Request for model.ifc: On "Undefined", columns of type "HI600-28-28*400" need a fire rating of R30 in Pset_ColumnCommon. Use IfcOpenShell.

First a look at what the model holds.

```python
import ifcopenshell
import ifcopenshell.util.element

model = ifcopenshell.open("model.ifc")
print(model.schema)
storey = next(s for s in model.by_type("IfcBuildingStorey") if s.Name == "Undefined")
columns = [e for e in ifcopenshell.util.element.get_decomposition(storey) if e.is_a("IfcColumn")]
seen = {}
for e in columns:
    element_type = ifcopenshell.util.element.get_type(e)
    key = (element_type.Name if element_type != e and element_type else None, ifcopenshell.util.element.get_pset(e, "Pset_ColumnCommon", "FireRating"))
    seen[key] = seen.get(key, 0) + 1
for (name, value), count in sorted(seen.items(), key=str):
    print(count, "x", name, "|", value)
```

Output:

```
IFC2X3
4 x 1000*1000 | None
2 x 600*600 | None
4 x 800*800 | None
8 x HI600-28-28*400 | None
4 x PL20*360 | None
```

```python
import ifcopenshell
import ifcopenshell.api.pset
import ifcopenshell.util.element

model = ifcopenshell.open("model.ifc")

storey = next(s for s in model.by_type("IfcBuildingStorey") if s.Name == "Undefined")
columns = [e for e in ifcopenshell.util.element.get_decomposition(storey) if e.is_a("IfcColumn")]

count = 0
for e in columns:
    element_type = ifcopenshell.util.element.get_type(e)
    if element_type in (None, e) or element_type.Name != "HI600-28-28*400":
        continue
    found = ifcopenshell.util.element.get_pset(e, "Pset_ColumnCommon", should_inherit=False)
    if found:
        pset = model.by_id(found["id"])
        if len(ifcopenshell.util.element.get_elements_by_pset(pset)) > 1:
            pset = ifcopenshell.api.pset.unshare_pset(model, products=[e], pset=pset)[0]
    else:
        pset = ifcopenshell.api.pset.add_pset(model, product=e, name="Pset_ColumnCommon")
    ifcopenshell.api.pset.edit_pset(model, pset=pset, properties={"FireRating": "R30"})
    count += 1

print(count, "columns updated")

model.write("model_edited.ifc")
```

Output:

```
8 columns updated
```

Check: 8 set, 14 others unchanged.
